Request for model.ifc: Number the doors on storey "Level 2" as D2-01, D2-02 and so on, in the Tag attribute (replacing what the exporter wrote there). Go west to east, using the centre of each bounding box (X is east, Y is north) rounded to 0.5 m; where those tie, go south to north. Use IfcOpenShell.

First a look at what the model holds.

```python
import ifcopenshell
import ifcopenshell.util.element
import ifcopenshell.util.placement

model = ifcopenshell.open("model.ifc")
print(model.schema)
storey = next(s for s in model.by_type("IfcBuildingStorey") if s.Name == "Level 2")
doors = [e for e in ifcopenshell.util.element.get_decomposition(storey) if e.is_a("IfcDoor")]
for e in sorted(doors, key=lambda e: e.id()):
    origin = ifcopenshell.util.placement.get_local_placement(e.ObjectPlacement)[:3, 3]
    print(e.id(), e.Tag, e.Name, origin.round(2) + 0.0, sep=" | ")
```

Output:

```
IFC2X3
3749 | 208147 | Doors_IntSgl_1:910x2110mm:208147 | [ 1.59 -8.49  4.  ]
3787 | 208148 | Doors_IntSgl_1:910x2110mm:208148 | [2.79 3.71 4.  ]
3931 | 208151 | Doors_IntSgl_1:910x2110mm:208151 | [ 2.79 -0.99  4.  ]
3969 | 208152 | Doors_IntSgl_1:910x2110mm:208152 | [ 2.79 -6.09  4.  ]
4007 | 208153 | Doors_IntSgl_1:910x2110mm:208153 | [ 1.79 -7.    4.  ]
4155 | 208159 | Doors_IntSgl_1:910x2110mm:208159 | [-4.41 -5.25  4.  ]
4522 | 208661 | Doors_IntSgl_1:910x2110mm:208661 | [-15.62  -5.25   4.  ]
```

```python
import ifcopenshell
import ifcopenshell.geom
import ifcopenshell.util.element
import ifcopenshell.util.shape

model = ifcopenshell.open("model.ifc")
settings = ifcopenshell.geom.settings()
settings.set("use-world-coords", True)


def centre(element):
    shape = ifcopenshell.geom.create_shape(settings, element)
    return ifcopenshell.util.shape.get_bbox_centroid(shape.geometry)


storey = next(s for s in model.by_type("IfcBuildingStorey") if s.Name == "Level 2")
doors = [e for e in ifcopenshell.util.element.get_decomposition(storey) if e.is_a("IfcDoor")]

# Insertion points can sit at a corner or the storey origin, so sort by the geometry (in metres).
centres = {e: centre(e) for e in doors}
doors.sort(key=lambda e: (round(centres[e][0] / 0.5), centres[e][1]))

for i, e in enumerate(doors, start=1):
    number = f"D2-{i:02d}"
    e.Tag = number
    print(e.id(), number)

model.write("model-out.ifc")
```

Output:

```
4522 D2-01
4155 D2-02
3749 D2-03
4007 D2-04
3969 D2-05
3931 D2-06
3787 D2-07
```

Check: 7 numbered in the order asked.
